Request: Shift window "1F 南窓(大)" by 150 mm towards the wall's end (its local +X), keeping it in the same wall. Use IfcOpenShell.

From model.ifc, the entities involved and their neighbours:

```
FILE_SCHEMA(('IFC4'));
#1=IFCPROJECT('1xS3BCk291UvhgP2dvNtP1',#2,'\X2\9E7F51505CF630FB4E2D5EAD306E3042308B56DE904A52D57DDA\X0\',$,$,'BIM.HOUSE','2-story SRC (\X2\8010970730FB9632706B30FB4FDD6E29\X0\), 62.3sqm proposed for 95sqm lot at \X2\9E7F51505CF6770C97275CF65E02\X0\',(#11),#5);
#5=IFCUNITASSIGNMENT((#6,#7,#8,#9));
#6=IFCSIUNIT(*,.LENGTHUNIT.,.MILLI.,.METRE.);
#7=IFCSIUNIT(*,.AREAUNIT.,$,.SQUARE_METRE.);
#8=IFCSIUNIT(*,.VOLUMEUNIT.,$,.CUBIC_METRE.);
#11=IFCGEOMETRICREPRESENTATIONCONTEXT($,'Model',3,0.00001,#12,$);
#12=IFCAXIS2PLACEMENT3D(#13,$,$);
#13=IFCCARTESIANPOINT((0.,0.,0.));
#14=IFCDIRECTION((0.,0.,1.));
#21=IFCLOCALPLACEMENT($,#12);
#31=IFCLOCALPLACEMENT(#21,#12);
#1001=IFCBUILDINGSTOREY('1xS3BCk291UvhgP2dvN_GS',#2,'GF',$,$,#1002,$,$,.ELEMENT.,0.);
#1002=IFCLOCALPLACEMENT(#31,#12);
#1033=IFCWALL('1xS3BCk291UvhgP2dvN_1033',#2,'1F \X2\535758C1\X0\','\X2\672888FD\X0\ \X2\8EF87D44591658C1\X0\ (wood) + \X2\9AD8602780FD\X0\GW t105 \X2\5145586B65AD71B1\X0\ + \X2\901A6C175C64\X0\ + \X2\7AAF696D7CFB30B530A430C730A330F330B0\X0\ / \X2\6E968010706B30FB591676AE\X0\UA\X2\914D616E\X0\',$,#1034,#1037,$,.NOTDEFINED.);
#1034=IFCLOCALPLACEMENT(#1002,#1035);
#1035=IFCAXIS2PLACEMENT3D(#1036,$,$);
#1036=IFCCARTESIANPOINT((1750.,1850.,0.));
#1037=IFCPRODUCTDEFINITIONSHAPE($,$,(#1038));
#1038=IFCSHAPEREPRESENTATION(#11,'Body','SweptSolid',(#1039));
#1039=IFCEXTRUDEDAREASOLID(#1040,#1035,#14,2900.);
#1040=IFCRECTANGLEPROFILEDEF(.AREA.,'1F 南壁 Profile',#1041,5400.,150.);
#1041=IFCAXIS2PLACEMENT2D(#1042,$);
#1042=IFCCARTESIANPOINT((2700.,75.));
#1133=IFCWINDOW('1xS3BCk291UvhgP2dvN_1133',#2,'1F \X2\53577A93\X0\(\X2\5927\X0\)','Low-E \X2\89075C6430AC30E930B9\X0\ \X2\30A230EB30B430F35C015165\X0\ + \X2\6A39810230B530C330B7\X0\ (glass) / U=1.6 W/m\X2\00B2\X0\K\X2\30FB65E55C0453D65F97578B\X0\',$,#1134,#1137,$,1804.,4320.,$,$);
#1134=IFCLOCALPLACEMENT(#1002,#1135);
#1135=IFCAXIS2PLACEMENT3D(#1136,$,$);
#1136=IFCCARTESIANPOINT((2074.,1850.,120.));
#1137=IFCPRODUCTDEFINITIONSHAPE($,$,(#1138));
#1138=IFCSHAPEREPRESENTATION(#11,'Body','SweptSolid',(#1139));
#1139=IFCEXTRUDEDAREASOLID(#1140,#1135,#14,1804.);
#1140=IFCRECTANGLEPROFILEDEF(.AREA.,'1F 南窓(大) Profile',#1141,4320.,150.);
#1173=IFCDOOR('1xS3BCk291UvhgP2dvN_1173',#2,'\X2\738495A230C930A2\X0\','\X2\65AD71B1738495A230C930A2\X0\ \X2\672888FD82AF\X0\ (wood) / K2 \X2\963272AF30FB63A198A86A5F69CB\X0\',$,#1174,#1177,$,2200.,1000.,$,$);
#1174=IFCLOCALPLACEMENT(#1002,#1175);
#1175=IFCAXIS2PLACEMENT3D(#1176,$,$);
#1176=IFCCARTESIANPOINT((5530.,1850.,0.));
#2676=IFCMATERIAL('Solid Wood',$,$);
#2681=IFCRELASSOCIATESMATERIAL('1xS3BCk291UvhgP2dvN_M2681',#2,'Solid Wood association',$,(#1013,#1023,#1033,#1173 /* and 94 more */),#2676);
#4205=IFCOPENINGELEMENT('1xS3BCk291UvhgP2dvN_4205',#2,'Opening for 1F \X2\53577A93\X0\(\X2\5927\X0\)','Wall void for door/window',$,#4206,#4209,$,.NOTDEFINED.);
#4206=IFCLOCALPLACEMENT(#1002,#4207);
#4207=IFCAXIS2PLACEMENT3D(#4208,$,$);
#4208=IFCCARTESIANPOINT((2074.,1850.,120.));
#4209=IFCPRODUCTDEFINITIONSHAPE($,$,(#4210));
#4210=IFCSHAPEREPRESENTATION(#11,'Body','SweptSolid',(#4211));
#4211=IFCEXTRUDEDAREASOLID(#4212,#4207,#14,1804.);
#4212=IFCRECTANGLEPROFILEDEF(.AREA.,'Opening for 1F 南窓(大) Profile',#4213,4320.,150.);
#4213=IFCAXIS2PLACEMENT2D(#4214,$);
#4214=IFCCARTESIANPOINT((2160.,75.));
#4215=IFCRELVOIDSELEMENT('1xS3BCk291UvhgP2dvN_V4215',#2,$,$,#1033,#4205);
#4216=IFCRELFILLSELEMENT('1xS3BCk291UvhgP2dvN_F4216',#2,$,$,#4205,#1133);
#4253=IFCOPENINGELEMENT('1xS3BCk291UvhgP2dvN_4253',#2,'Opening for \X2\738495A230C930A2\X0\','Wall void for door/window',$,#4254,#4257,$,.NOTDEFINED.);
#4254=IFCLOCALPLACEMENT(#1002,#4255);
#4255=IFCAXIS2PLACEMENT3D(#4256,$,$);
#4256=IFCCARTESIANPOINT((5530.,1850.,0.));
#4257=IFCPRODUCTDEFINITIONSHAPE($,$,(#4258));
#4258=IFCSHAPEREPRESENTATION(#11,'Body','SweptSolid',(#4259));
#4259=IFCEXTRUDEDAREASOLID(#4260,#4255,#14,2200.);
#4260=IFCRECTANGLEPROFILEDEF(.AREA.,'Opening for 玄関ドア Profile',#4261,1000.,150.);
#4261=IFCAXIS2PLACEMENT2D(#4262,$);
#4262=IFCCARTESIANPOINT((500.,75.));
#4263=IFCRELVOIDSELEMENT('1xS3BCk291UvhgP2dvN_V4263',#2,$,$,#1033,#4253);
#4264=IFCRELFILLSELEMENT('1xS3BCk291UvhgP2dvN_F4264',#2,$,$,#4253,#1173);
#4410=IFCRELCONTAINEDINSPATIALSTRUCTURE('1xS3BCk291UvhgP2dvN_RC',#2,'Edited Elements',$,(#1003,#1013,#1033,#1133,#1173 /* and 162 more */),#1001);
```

```python
import ifcopenshell
import ifcopenshell.api.geometry
import ifcopenshell.util.placement
import ifcopenshell.util.unit

model = ifcopenshell.open("model.ifc")
unit_scale = ifcopenshell.util.unit.calculate_unit_scale(model)

window = model.by_guid("1xS3BCk291UvhgP2dvN_1133")
opening = window.FillsVoids[0].RelatingOpeningElement
wall = opening.VoidsElements[0].RelatingBuildingElement

wall_matrix = ifcopenshell.util.placement.get_local_placement(wall.ObjectPlacement)
shift = wall_matrix[:3, 0] * 0.15 / unit_scale
before = ifcopenshell.util.placement.get_local_placement(window.ObjectPlacement)[:3, 3].copy()

# The window is not placed relative to its opening, so move both.
for product in (opening, window):
    matrix = ifcopenshell.util.placement.get_local_placement(product.ObjectPlacement)
    matrix[:3, 3] += shift
    ifcopenshell.api.geometry.edit_object_placement(model, product=product, matrix=matrix, is_si=False)

after = ifcopenshell.util.placement.get_local_placement(window.ObjectPlacement)[:3, 3]
print("window moved by", (after - before).round(3) + 0.0)

model.write("model_rev.ifc")
```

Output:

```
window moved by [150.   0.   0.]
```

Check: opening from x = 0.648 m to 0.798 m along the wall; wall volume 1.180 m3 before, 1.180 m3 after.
